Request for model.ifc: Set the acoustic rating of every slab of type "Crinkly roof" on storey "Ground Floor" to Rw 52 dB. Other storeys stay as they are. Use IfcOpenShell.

First a look at what the model holds.

```python
import ifcopenshell
import ifcopenshell.util.element

model = ifcopenshell.open("model.ifc")
print(model.schema)
storey = next(s for s in model.by_type("IfcBuildingStorey") if s.Name == "Ground Floor")
slabs = [e for e in ifcopenshell.util.element.get_decomposition(storey) if e.is_a("IfcSlab")]
seen = {}
for e in slabs:
    element_type = ifcopenshell.util.element.get_type(e)
    key = (element_type.Name if element_type != e and element_type else None, ifcopenshell.util.element.get_pset(e, "Pset_SlabCommon", "AcousticRating"))
    seen[key] = seen.get(key, 0) + 1
for (name, value), count in sorted(seen.items(), key=str):
    print(count, "x", name, "|", value)
```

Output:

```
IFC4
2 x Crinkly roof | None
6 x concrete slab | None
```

```python
import ifcopenshell
import ifcopenshell.api.pset
import ifcopenshell.util.element

model = ifcopenshell.open("model.ifc")

storey = next(s for s in model.by_type("IfcBuildingStorey") if s.Name == "Ground Floor")
slabs = [e for e in ifcopenshell.util.element.get_decomposition(storey) if e.is_a("IfcSlab")]

count = 0
for e in slabs:
    element_type = ifcopenshell.util.element.get_type(e)
    if element_type in (None, e) or element_type.Name != "Crinkly roof":
        continue
    # add_pset returns the element's existing set when there is one.
    pset = ifcopenshell.api.pset.add_pset(model, product=e, name="Pset_SlabCommon")
    ifcopenshell.api.pset.edit_pset(model, pset=pset, properties={"AcousticRating": "Rw 52 dB"})
    count += 1

print(count, "slabs updated")

model.write("model_edited.ifc")
```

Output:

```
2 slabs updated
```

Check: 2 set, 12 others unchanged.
